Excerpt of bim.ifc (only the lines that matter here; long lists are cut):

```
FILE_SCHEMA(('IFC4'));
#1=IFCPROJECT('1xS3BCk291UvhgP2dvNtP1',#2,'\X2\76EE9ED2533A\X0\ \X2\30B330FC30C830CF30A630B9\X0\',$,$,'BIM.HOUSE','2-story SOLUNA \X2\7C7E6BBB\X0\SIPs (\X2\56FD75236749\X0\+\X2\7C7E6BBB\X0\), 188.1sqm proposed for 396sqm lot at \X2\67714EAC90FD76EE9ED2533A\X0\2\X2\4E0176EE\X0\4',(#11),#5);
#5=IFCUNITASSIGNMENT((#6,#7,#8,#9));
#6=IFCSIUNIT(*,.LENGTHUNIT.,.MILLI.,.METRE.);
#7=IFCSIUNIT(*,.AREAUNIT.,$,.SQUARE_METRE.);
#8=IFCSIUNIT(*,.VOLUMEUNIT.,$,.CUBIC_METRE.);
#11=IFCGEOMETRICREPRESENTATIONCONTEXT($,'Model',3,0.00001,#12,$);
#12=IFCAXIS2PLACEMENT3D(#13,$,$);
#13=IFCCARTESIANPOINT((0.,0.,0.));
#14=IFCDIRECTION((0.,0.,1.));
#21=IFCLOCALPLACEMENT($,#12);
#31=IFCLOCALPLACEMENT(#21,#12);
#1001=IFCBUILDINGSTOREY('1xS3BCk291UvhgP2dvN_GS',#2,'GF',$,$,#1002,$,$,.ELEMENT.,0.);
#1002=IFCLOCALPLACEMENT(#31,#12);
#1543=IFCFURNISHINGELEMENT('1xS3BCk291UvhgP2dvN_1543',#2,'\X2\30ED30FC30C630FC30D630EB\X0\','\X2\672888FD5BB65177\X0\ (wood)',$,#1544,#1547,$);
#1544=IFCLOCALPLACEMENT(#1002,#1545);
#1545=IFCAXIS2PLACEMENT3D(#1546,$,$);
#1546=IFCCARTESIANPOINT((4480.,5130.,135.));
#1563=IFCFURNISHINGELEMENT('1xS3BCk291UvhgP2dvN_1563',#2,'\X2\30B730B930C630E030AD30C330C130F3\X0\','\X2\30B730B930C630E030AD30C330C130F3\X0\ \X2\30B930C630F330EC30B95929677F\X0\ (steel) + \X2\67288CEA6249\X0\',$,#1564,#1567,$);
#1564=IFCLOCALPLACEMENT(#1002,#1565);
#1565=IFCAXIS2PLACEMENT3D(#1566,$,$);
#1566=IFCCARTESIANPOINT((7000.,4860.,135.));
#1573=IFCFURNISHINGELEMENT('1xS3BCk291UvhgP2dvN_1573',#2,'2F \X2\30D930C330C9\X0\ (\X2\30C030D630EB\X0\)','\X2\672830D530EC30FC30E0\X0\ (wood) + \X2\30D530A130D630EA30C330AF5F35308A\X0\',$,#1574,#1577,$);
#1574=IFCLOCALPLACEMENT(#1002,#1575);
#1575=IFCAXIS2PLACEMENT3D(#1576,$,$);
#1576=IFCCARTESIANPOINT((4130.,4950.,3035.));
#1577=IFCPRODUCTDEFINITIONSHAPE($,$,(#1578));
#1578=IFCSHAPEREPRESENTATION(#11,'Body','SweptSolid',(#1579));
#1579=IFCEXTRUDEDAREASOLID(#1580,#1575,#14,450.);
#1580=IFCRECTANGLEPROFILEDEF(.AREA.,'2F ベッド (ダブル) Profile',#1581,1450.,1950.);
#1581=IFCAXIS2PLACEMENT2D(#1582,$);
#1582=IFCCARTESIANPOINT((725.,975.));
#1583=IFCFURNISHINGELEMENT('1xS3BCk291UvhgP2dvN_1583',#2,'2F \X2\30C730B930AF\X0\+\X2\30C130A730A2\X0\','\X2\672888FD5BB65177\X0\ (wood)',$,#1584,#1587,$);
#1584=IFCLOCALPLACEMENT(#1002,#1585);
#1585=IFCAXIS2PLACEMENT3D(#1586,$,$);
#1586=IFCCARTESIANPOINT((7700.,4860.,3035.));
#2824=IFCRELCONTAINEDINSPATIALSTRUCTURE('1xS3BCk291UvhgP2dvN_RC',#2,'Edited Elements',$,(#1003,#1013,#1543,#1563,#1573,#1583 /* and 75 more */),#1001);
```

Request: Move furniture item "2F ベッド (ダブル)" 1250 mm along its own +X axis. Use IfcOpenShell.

```python
import ifcopenshell
import ifcopenshell.api.geometry
import ifcopenshell.util.placement

model = ifcopenshell.open("bim.ifc")

item = model.by_id(1573)
matrix = ifcopenshell.util.placement.get_local_placement(item.ObjectPlacement)
matrix[:3, 3] += matrix[:3, 0] * 1250.0
ifcopenshell.api.geometry.edit_object_placement(model, product=item, matrix=matrix, is_si=False)

print(ifcopenshell.util.placement.get_local_placement(item.ObjectPlacement).round(3) + 0.0)

model.write("bim_edited.ifc")
```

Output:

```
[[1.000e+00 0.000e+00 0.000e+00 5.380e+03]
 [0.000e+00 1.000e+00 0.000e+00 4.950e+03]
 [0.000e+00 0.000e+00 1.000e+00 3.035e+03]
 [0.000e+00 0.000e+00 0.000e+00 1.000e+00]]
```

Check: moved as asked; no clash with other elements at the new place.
